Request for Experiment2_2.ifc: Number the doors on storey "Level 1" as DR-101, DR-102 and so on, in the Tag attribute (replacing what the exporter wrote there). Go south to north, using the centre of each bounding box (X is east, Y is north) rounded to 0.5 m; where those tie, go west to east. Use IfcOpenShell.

First a look at what the model holds.

```python
import ifcopenshell
import ifcopenshell.util.element
import ifcopenshell.util.placement

model = ifcopenshell.open("Experiment2_2.ifc")
print(model.schema)
storey = next(s for s in model.by_type("IfcBuildingStorey") if s.Name == "Level 1")
doors = [e for e in ifcopenshell.util.element.get_decomposition(storey) if e.is_a("IfcDoor")]
for e in sorted(doors, key=lambda e: e.id()):
    origin = ifcopenshell.util.placement.get_local_placement(e.ObjectPlacement)[:3, 3]
    print(e.id(), e.Tag, e.Name, origin.round(2) + 0.0, sep=" | ")
```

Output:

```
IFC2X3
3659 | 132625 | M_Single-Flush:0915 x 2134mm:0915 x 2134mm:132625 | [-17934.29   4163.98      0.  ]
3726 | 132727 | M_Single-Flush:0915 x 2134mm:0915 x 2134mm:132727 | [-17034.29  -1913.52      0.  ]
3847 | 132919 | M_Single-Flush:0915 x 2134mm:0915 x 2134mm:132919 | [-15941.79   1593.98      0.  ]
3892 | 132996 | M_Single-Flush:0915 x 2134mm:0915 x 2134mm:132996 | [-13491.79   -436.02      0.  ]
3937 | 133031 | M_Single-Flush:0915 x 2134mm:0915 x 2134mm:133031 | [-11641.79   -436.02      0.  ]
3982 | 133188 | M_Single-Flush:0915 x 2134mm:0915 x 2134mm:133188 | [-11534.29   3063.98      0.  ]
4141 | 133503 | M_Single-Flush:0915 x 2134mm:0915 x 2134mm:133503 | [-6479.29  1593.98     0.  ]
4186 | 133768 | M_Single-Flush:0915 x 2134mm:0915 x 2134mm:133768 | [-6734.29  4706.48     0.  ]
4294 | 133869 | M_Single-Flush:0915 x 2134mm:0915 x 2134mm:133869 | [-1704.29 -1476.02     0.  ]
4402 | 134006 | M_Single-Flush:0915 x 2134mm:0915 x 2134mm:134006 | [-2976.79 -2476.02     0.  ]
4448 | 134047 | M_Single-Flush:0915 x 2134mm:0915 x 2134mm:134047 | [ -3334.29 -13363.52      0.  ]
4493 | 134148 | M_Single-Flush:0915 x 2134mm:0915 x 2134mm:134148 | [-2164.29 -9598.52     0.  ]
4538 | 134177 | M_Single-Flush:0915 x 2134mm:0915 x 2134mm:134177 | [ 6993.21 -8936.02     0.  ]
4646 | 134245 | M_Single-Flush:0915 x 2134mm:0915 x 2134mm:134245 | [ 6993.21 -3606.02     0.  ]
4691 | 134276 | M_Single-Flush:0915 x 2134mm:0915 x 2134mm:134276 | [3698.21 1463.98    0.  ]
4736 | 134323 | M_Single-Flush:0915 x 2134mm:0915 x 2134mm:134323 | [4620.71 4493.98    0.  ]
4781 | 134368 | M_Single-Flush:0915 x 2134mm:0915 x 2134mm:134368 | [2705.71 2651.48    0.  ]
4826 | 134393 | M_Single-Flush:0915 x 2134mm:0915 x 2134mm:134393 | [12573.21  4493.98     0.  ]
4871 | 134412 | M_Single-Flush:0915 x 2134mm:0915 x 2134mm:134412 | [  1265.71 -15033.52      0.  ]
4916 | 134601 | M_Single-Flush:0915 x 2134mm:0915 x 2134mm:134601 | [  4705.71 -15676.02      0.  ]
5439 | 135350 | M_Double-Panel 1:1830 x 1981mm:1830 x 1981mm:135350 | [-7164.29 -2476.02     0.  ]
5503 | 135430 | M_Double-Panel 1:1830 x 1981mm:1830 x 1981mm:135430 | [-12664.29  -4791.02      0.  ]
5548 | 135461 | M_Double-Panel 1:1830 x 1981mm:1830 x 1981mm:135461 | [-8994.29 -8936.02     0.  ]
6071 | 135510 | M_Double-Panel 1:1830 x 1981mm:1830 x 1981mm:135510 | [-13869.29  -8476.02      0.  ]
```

```python
import ifcopenshell
import ifcopenshell.geom
import ifcopenshell.util.element
import ifcopenshell.util.shape

model = ifcopenshell.open("Experiment2_2.ifc")
settings = ifcopenshell.geom.settings()
settings.set("use-world-coords", True)


def centre(element):
    shape = ifcopenshell.geom.create_shape(settings, element)
    return ifcopenshell.util.shape.get_bbox_centroid(shape.geometry)


storey = next(s for s in model.by_type("IfcBuildingStorey") if s.Name == "Level 1")
doors = [e for e in ifcopenshell.util.element.get_decomposition(storey) if e.is_a("IfcDoor")]

# Insertion points can sit at a corner or the storey origin, so sort by the geometry (in metres).
centres = {e: centre(e) for e in doors}
doors.sort(key=lambda e: (round(centres[e][1] / 0.5), centres[e][0]))

for i, e in enumerate(doors, start=1):
    number = f"DR-1{i:02d}"
    e.Tag = number
    print(e.id(), number)

model.write("Experiment2_2_v2.ifc")
```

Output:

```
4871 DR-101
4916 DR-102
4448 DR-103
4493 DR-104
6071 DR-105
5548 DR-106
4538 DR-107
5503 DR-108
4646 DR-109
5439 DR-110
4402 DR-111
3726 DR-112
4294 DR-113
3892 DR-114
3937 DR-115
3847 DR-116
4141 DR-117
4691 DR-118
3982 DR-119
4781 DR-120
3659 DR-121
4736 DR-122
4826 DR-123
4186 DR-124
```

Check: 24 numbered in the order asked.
